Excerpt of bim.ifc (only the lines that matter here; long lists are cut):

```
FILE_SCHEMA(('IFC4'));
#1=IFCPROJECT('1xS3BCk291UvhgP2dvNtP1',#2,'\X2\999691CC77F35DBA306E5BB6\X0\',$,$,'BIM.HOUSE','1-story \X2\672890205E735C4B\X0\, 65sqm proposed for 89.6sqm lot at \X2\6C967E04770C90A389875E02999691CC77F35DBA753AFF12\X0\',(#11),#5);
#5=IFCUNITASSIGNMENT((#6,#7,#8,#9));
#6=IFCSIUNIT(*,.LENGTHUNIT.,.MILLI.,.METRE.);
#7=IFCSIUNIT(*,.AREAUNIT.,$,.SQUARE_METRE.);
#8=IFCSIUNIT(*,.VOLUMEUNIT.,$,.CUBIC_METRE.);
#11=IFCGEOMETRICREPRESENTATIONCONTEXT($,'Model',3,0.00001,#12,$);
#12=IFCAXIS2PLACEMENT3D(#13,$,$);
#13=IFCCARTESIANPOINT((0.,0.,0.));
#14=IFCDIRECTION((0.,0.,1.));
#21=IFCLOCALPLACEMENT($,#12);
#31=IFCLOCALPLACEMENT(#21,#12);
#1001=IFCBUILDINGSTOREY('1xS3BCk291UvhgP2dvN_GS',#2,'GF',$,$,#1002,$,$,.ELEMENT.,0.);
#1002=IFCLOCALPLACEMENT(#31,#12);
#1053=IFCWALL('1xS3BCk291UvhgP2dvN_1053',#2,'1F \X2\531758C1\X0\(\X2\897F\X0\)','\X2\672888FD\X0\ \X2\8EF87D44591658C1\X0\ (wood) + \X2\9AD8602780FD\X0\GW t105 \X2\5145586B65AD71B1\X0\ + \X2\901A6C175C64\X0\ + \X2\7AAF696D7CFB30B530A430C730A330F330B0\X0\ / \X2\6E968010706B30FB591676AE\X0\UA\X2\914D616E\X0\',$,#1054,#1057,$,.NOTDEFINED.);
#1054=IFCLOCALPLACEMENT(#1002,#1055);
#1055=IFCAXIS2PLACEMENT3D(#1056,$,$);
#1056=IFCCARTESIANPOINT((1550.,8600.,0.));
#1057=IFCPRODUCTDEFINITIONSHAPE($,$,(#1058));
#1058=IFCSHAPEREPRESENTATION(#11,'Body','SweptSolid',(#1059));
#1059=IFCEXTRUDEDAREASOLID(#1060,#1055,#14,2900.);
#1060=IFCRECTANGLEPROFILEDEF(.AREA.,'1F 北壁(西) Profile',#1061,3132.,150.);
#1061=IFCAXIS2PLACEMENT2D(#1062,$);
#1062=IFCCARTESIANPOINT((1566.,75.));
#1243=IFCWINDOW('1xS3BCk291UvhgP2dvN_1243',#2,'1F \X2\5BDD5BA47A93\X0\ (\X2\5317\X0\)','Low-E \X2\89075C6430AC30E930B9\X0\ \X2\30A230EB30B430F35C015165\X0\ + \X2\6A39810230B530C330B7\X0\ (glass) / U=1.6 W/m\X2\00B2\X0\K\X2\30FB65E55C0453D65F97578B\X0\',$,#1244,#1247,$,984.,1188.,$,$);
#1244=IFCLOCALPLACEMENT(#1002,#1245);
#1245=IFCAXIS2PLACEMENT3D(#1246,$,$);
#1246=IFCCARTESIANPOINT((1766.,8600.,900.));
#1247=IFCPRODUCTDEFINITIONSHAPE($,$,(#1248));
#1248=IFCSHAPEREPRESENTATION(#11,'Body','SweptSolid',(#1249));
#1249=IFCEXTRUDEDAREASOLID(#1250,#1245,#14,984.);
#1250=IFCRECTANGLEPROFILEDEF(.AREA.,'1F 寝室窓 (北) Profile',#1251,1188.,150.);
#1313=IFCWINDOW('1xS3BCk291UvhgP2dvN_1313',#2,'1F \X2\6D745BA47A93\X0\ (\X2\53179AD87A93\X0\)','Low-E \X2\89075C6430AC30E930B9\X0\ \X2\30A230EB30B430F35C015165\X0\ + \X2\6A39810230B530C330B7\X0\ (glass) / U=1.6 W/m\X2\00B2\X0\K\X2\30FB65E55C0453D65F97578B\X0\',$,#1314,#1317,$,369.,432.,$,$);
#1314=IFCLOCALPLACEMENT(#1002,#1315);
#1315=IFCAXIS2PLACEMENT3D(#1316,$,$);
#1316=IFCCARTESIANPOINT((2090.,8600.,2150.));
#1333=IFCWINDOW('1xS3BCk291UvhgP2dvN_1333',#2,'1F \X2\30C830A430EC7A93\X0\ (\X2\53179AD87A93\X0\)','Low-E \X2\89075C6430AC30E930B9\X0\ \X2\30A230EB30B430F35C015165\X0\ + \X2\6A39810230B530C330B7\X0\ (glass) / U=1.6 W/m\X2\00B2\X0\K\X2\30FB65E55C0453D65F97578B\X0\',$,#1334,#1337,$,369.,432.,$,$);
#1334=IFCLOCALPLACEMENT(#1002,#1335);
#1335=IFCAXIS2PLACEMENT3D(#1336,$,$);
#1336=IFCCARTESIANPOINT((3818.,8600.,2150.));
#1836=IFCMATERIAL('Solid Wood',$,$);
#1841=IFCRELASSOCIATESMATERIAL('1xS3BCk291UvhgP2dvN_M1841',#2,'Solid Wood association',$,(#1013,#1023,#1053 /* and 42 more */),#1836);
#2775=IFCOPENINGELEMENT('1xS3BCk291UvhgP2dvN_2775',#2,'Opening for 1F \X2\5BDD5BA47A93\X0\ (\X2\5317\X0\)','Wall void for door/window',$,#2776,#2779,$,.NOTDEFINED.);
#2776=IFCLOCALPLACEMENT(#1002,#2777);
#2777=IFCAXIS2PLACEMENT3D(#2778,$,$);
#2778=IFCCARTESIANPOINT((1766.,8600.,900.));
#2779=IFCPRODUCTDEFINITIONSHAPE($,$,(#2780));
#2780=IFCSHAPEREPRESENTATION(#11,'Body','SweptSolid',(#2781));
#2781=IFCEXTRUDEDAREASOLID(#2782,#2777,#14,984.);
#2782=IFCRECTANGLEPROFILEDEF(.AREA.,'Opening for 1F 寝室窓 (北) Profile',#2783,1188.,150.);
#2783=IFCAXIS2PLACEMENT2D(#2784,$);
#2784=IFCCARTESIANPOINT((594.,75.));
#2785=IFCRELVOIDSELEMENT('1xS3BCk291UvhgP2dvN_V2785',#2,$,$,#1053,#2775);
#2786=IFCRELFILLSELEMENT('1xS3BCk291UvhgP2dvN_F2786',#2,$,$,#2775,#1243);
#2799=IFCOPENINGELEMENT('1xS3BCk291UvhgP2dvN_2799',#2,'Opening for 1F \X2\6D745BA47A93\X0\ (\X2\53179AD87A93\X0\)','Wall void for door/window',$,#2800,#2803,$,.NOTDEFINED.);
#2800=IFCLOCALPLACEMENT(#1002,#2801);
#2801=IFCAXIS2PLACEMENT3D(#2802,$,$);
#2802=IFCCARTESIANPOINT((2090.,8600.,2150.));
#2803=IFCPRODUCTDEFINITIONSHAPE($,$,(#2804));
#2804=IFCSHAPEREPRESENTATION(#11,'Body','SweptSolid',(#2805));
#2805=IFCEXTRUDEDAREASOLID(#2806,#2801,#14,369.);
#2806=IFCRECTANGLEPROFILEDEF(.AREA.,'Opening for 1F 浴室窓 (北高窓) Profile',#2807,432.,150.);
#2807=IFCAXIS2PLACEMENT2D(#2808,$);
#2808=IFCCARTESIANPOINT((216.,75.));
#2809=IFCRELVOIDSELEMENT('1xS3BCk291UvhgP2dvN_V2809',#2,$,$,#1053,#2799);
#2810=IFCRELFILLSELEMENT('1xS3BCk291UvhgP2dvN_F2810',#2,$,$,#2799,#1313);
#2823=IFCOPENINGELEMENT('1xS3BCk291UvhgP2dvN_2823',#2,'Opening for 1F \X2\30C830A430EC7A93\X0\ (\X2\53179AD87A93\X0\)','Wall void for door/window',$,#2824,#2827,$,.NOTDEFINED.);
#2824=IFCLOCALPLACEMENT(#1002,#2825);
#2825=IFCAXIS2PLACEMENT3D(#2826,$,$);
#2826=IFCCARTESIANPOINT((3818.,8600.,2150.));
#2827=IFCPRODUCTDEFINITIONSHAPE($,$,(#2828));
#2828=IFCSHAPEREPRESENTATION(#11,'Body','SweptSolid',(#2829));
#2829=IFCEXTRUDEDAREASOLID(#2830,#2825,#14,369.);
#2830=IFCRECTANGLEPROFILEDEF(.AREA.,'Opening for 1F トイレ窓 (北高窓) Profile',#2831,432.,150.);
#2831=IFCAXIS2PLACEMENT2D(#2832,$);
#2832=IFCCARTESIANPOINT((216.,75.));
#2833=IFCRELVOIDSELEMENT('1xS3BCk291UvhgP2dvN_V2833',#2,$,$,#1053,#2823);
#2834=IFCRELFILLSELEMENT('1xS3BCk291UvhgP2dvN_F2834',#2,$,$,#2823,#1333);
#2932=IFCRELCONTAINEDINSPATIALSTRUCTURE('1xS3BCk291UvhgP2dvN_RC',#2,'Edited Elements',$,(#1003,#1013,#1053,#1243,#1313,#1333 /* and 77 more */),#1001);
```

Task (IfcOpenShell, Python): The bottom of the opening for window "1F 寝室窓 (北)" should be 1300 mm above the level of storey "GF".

```python
import numpy as np
import ifcopenshell
import ifcopenshell.api.geometry
import ifcopenshell.geom
import ifcopenshell.util.element
import ifcopenshell.util.placement
import ifcopenshell.util.shape
import ifcopenshell.util.unit

model = ifcopenshell.open("bim.ifc")
unit_scale = ifcopenshell.util.unit.calculate_unit_scale(model)

window = model.by_guid("1xS3BCk291UvhgP2dvN_1243")
opening = window.FillsVoids[0].RelatingOpeningElement
storey = ifcopenshell.util.element.get_container(window, ifc_class="IfcBuildingStorey")
level = ifcopenshell.util.placement.get_local_placement(storey.ObjectPlacement)[2, 3]

# The opening's origin need not be at the sill, so measure its lowest point.
shape = ifcopenshell.geom.create_shape(ifcopenshell.geom.settings(), opening)
bottom = ifcopenshell.util.shape.get_shape_bottom_elevation(shape, shape.geometry) / unit_scale
dz = level + 1.3 / unit_scale - bottom

shift = np.array([0.0, 0.0, dz])
# The window is not placed relative to its opening, so move both.
for product in (opening, window):
    matrix = ifcopenshell.util.placement.get_local_placement(product.ObjectPlacement)
    matrix[:3, 3] += shift
    ifcopenshell.api.geometry.edit_object_placement(model, product=product, matrix=matrix, is_si=False)

print(f"moved by {dz * unit_scale:+.3f} m")

model.write("bim_edited.ifc")
```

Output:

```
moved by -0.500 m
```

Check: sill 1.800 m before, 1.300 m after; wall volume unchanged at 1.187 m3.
